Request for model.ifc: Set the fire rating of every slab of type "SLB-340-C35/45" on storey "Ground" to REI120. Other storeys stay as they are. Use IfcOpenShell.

First a look at what the model holds.

```python
import ifcopenshell
import ifcopenshell.util.element

model = ifcopenshell.open("model.ifc")
print(model.schema)
storey = next(s for s in model.by_type("IfcBuildingStorey") if s.Name == "Ground")
slabs = [e for e in ifcopenshell.util.element.get_decomposition(storey) if e.is_a("IfcSlab")]
seen = {}
for e in slabs:
    element_type = ifcopenshell.util.element.get_type(e)
    key = (element_type.Name if element_type != e and element_type else None, ifcopenshell.util.element.get_pset(e, "Pset_SlabCommon", "FireRating"))
    seen[key] = seen.get(key, 0) + 1
for (name, value), count in sorted(seen.items(), key=str):
    print(count, "x", name, "|", value)
```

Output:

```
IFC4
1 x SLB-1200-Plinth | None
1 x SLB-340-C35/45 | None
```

```python
import ifcopenshell
import ifcopenshell.api.pset
import ifcopenshell.util.element

model = ifcopenshell.open("model.ifc")

storey = next(s for s in model.by_type("IfcBuildingStorey") if s.Name == "Ground")
slabs = [e for e in ifcopenshell.util.element.get_decomposition(storey) if e.is_a("IfcSlab")]

count = 0
for e in slabs:
    element_type = ifcopenshell.util.element.get_type(e)
    if element_type in (None, e) or element_type.Name != "SLB-340-C35/45":
        continue
    # add_pset returns the element's existing set when there is one.
    pset = ifcopenshell.api.pset.add_pset(model, product=e, name="Pset_SlabCommon")
    ifcopenshell.api.pset.edit_pset(model, pset=pset, properties={"FireRating": "REI120"})
    count += 1

print(count, "slabs updated")

model.write("model-out.ifc")
```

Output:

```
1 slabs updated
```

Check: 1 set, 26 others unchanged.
